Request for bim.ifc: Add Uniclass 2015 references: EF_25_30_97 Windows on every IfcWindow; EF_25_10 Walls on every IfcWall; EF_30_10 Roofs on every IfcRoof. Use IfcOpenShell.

First a look at what the model holds.

```python
import ifcopenshell

model = ifcopenshell.open("bim.ifc")
print(model.schema)
print("classifications:", [c.Name for c in model.by_type("IfcClassification")])
for ifc_class in ("IfcDoor", "IfcRoof", "IfcStair", "IfcWall", "IfcWindow"):
    print(ifc_class, len(model.by_type(ifc_class)))
```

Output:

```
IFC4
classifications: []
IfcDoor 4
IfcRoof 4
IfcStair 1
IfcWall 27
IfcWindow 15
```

```python
import ifcopenshell
import ifcopenshell.api.classification

model = ifcopenshell.open("bim.ifc")

system = ifcopenshell.api.classification.add_classification(model, classification="Uniclass 2015")

codes = {
    "IfcWindow": ("EF_25_30_97", "Windows"),
    "IfcWall": ("EF_25_10", "Walls"),
    "IfcRoof": ("EF_30_10", "Roofs"),
}
for ifc_class, (code, name) in codes.items():
    products = model.by_type(ifc_class)
    ifcopenshell.api.classification.add_reference(
        model, products=products, classification=system, identification=code, name=name
    )
    print(code, len(products))

model.write("bim_edited.ifc")
```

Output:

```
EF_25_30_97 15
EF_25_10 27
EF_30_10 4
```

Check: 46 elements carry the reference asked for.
